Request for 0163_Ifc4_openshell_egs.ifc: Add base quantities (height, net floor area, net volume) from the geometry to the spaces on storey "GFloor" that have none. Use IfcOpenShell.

First a look at what the model holds.

```python
import ifcopenshell
import ifcopenshell.util.element
import ifcopenshell.util.unit

model = ifcopenshell.open("0163_Ifc4_openshell_egs.ifc")
print(model.schema)
for unit_type in ("LENGTHUNIT", "AREAUNIT", "VOLUMEUNIT"):
    print(unit_type, ifcopenshell.util.unit.calculate_unit_scale(model, unit_type))
storey = next(s for s in model.by_type("IfcBuildingStorey") if s.Name == "GFloor")
spaces = [e for e in ifcopenshell.util.element.get_decomposition(storey) if e.is_a("IfcSpace")]
for e in sorted(spaces, key=lambda e: e.id()):
    print(e.id(), e.is_a(), e.Name, list(ifcopenshell.util.element.get_psets(e, qtos_only=True)), sep=" | ")
```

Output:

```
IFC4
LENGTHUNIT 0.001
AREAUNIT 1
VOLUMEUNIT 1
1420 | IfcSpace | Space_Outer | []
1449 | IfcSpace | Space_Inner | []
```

```python
import ifcopenshell
import ifcopenshell.api.pset
import ifcopenshell.geom
import ifcopenshell.util.element
import ifcopenshell.util.shape
import ifcopenshell.util.unit

model = ifcopenshell.open("0163_Ifc4_openshell_egs.ifc")
unit_scale = ifcopenshell.util.unit.calculate_unit_scale(model)
area_scale = ifcopenshell.util.unit.calculate_unit_scale(model, "AREAUNIT")
volume_scale = ifcopenshell.util.unit.calculate_unit_scale(model, "VOLUMEUNIT")
settings = ifcopenshell.geom.settings()

storey = next(s for s in model.by_type("IfcBuildingStorey") if s.Name == "GFloor")
spaces = [e for e in ifcopenshell.util.element.get_decomposition(storey) if e.is_a("IfcSpace")]

for e in sorted(spaces, key=lambda e: e.id()):
    if ifcopenshell.util.element.get_psets(e, qtos_only=True, should_inherit=False):
        continue
    # Geometry comes back in metres, in the element's own axes.
    shape = ifcopenshell.geom.create_shape(settings, e)
    values = {
        "Height": ifcopenshell.util.shape.get_z(shape.geometry) / unit_scale,
        "NetFloorArea": ifcopenshell.util.shape.get_footprint_area(shape.geometry) / area_scale,
        "NetVolume": ifcopenshell.util.shape.get_volume(shape.geometry) / volume_scale,
    }
    qto = ifcopenshell.api.pset.add_qto(model, product=e, name="Qto_SpaceBaseQuantities")
    ifcopenshell.api.pset.edit_qto(model, qto=qto, properties=values)
    print(e.id(), {k: round(v, 3) for k, v in values.items()})

model.write("0163_Ifc4_openshell_egs_updated.ifc")
```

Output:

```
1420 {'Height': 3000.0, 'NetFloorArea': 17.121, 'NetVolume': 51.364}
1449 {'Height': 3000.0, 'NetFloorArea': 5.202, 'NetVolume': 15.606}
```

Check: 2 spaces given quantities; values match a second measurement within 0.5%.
